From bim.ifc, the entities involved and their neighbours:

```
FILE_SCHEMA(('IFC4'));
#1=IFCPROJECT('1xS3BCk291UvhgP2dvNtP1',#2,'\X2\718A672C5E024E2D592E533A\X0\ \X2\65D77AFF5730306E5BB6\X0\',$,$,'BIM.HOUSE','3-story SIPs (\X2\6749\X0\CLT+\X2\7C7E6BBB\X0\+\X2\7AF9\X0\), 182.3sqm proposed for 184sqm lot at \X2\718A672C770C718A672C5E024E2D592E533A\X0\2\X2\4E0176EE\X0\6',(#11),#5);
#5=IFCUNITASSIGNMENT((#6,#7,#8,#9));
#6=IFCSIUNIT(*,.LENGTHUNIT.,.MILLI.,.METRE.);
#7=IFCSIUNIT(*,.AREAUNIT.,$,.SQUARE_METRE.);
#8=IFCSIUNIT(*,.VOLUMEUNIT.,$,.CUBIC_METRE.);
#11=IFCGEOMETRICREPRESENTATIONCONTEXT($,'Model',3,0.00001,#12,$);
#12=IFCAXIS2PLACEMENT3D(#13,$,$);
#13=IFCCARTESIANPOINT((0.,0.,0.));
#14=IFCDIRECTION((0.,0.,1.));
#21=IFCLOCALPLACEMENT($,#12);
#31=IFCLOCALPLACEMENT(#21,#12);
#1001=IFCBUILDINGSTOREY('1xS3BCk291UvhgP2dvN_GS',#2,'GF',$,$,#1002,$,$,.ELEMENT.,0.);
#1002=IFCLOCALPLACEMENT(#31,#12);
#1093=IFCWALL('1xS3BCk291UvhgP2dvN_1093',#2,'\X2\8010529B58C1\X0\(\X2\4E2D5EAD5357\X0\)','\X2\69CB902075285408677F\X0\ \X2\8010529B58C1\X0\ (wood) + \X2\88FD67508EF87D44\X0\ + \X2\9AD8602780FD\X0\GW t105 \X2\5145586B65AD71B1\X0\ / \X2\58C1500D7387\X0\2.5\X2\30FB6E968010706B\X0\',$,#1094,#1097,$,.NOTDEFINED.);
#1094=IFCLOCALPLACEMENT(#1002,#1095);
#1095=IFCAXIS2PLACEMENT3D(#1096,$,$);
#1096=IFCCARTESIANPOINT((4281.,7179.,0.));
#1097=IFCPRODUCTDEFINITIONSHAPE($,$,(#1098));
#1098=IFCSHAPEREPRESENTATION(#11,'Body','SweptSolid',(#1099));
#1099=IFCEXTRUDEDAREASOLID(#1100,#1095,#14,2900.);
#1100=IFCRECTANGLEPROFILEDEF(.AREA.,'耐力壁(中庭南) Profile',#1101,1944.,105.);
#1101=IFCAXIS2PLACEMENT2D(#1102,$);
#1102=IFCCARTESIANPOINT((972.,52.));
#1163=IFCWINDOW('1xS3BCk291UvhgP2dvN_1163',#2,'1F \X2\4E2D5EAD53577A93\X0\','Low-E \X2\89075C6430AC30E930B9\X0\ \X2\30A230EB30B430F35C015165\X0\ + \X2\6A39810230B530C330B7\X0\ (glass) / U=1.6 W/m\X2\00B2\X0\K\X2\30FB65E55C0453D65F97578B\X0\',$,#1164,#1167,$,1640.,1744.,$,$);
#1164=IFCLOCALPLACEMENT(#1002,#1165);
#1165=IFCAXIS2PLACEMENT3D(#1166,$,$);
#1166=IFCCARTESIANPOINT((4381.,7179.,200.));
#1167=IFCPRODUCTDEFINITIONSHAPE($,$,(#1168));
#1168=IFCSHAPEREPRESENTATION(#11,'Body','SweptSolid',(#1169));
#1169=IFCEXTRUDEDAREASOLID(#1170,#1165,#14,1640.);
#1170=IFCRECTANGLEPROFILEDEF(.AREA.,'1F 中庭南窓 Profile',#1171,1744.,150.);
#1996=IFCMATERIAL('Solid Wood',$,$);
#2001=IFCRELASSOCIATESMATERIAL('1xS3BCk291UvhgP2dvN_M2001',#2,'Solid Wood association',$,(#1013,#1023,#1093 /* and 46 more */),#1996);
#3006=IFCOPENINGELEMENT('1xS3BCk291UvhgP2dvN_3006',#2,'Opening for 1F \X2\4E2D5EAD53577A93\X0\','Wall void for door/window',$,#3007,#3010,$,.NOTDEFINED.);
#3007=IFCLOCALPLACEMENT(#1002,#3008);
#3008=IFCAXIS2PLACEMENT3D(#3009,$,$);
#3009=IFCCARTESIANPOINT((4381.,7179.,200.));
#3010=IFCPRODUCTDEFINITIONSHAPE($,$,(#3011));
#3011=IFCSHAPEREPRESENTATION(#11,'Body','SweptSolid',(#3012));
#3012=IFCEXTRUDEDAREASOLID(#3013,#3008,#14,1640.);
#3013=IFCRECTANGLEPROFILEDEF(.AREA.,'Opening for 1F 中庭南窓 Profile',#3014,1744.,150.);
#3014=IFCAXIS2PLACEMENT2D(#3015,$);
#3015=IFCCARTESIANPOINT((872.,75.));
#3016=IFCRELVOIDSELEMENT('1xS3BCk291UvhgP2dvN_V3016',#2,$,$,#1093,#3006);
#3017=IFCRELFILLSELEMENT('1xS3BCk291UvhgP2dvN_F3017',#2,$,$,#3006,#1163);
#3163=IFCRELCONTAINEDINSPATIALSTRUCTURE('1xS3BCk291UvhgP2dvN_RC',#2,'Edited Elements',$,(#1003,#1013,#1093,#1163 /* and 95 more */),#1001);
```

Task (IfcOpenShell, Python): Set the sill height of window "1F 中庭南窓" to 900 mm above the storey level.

```python
import numpy as np
import ifcopenshell
import ifcopenshell.api.geometry
import ifcopenshell.geom
import ifcopenshell.util.element
import ifcopenshell.util.placement
import ifcopenshell.util.shape
import ifcopenshell.util.unit

model = ifcopenshell.open("bim.ifc")
unit_scale = ifcopenshell.util.unit.calculate_unit_scale(model)

window = model.by_guid("1xS3BCk291UvhgP2dvN_1163")
opening = window.FillsVoids[0].RelatingOpeningElement
storey = ifcopenshell.util.element.get_container(window, ifc_class="IfcBuildingStorey")
level = ifcopenshell.util.placement.get_local_placement(storey.ObjectPlacement)[2, 3]

# The opening's origin need not be at the sill, so measure its lowest point.
shape = ifcopenshell.geom.create_shape(ifcopenshell.geom.settings(), opening)
bottom = ifcopenshell.util.shape.get_shape_bottom_elevation(shape, shape.geometry) / unit_scale
dz = level + 0.9 / unit_scale - bottom

shift = np.array([0.0, 0.0, dz])
# The window is not placed relative to its opening, so move both.
for product in (opening, window):
    matrix = ifcopenshell.util.placement.get_local_placement(product.ObjectPlacement)
    matrix[:3, 3] += shift
    ifcopenshell.api.geometry.edit_object_placement(model, product=product, matrix=matrix, is_si=False)

print(f"moved by {dz * unit_scale:+.3f} m")

model.write("bim-out.ifc")
```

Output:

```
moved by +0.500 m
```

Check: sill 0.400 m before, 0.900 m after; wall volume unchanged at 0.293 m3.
